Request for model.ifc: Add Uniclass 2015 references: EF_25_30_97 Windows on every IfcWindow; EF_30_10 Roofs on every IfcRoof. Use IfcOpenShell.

First a look at what the model holds.

```python
import ifcopenshell

model = ifcopenshell.open("model.ifc")
print(model.schema)
print("classifications:", [c.Name for c in model.by_type("IfcClassification")])
for ifc_class in ("IfcDoor", "IfcRoof", "IfcStair", "IfcWall", "IfcWindow"):
    print(ifc_class, len(model.by_type(ifc_class)))
```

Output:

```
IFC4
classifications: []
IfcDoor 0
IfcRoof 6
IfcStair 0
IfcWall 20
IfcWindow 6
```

```python
import ifcopenshell
import ifcopenshell.api.classification

model = ifcopenshell.open("model.ifc")

system = ifcopenshell.api.classification.add_classification(model, classification="Uniclass 2015")

codes = {
    "IfcWindow": ("EF_25_30_97", "Windows"),
    "IfcRoof": ("EF_30_10", "Roofs"),
}
for ifc_class, (code, name) in codes.items():
    products = model.by_type(ifc_class)
    ifcopenshell.api.classification.add_reference(
        model, products=products, classification=system, identification=code, name=name
    )
    print(code, len(products))

model.write("model_edited.ifc")
```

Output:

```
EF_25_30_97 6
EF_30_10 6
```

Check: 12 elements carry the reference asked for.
